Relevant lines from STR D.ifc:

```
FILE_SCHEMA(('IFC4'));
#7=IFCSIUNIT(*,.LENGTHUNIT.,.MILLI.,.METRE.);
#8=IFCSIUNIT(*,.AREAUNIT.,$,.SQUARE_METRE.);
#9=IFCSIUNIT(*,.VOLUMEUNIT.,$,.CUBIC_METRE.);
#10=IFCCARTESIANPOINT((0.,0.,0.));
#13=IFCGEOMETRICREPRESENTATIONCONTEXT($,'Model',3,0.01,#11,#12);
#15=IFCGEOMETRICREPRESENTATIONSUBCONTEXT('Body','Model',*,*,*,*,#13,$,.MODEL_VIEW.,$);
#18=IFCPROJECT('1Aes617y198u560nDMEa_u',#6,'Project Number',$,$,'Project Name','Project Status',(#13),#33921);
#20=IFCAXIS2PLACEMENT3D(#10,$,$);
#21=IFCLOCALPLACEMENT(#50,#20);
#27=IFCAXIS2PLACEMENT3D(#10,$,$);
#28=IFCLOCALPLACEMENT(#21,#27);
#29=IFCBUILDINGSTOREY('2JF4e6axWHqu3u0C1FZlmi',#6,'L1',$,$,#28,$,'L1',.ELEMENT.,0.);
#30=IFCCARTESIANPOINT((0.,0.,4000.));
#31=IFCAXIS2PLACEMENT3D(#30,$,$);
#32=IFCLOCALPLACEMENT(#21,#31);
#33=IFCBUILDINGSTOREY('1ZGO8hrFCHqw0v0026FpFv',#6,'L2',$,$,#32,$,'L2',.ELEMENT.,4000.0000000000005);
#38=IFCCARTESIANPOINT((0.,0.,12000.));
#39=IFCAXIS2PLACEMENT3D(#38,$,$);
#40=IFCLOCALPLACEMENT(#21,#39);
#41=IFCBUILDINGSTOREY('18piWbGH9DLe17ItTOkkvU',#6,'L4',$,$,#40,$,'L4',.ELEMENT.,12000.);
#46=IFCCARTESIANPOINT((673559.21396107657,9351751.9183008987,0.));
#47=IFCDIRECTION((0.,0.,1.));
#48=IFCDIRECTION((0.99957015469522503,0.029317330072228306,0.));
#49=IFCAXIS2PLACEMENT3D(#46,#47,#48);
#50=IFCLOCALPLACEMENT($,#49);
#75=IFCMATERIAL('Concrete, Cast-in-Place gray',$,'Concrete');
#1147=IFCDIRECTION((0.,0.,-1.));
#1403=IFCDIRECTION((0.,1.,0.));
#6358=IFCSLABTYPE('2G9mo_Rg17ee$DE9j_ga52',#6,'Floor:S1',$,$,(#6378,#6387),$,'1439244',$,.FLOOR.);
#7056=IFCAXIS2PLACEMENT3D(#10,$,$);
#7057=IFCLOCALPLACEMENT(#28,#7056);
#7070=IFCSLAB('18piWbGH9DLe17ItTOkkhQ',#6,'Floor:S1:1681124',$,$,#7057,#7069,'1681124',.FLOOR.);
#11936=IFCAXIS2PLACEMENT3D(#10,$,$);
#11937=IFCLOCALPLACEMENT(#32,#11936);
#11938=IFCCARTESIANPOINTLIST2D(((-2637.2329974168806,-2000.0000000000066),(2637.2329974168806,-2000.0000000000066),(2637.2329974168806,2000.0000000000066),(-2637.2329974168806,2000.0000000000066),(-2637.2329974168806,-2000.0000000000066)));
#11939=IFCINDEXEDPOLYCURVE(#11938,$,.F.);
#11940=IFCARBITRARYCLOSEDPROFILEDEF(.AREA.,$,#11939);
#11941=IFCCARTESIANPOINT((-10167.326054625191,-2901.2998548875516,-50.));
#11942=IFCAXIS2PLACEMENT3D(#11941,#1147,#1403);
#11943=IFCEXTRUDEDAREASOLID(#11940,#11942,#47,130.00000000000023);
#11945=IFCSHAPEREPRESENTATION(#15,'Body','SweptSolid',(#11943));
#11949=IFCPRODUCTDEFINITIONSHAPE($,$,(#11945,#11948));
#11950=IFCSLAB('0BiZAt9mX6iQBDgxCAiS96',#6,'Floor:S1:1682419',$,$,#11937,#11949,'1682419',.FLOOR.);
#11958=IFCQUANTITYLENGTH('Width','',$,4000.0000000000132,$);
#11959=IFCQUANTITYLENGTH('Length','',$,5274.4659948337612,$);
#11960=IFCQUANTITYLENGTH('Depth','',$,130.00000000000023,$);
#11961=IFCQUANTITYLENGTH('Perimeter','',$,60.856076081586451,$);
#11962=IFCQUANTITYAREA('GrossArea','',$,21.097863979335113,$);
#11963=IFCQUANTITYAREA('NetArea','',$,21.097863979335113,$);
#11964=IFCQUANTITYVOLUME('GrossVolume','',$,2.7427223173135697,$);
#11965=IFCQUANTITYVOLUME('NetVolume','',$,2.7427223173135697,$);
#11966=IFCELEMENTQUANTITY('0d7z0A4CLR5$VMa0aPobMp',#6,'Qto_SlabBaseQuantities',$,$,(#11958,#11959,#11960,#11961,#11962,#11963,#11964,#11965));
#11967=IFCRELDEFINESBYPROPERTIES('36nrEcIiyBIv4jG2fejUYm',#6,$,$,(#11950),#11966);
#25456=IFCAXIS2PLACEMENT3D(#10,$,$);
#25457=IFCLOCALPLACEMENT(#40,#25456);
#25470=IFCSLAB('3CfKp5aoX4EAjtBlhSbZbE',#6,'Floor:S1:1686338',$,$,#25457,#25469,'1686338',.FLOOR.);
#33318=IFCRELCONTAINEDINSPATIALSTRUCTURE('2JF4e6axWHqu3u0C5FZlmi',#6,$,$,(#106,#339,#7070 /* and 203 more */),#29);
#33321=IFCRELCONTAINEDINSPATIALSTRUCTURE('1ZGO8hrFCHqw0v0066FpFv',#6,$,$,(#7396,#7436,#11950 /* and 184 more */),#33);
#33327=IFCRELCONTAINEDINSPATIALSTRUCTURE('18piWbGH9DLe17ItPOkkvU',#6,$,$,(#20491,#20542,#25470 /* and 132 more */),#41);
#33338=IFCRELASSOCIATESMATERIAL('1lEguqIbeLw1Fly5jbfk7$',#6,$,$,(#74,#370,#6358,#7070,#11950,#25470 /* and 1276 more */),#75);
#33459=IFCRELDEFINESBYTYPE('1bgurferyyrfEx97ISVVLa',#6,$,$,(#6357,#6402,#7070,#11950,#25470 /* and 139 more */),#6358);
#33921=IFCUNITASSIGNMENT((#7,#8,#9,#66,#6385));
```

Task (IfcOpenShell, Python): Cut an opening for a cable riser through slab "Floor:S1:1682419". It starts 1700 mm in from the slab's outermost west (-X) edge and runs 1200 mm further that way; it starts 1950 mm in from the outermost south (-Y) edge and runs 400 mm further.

```python
import numpy as np
import ifcopenshell
import ifcopenshell.api.feature
import ifcopenshell.api.geometry
import ifcopenshell.api.pset
import ifcopenshell.api.root
import ifcopenshell.geom
import ifcopenshell.util.element
import ifcopenshell.util.placement
import ifcopenshell.util.representation
import ifcopenshell.util.shape
import ifcopenshell.util.unit

model = ifcopenshell.open("STR D.ifc")
unit_scale = ifcopenshell.util.unit.calculate_unit_scale(model)
area_scale = ifcopenshell.util.unit.calculate_unit_scale(model, "AREAUNIT")
volume_scale = ifcopenshell.util.unit.calculate_unit_scale(model, "VOLUMEUNIT")
settings = ifcopenshell.geom.settings()


def volume(element):
    """Net volume in cubic metres, openings subtracted."""
    shape = ifcopenshell.geom.create_shape(settings, element)
    return ifcopenshell.util.shape.get_volume(shape.geometry)


slab = model.by_id(11950)
before = volume(slab)

# Extent in the slab's own axes, in metres. The edges named are its -X and -Y sides.
slab_shape = ifcopenshell.geom.create_shape(settings, slab)
vertices = ifcopenshell.util.shape.get_vertices(slab_shape.geometry)
x_min, y_min, bottom = vertices.min(axis=0)
top = vertices[:, 2].max()

opening = ifcopenshell.api.root.create_entity(model, ifc_class="IfcOpeningElement", name="Cable riser opening", predefined_type="OPENING")
context = ifcopenshell.util.representation.get_context(model, "Model", "Body", "MODEL_VIEW")
width, depth = 1.2, 0.4
outline = [(0.0, 0.0), (width, 0.0), (width, depth), (0.0, depth), (0.0, 0.0)]
# Overshoot both faces by 50 mm so the cut is clean.
shape = ifcopenshell.api.geometry.add_slab_representation(
    model, context=context, depth=top - bottom + 0.1, polyline=outline
)
ifcopenshell.api.geometry.assign_representation(model, product=opening, representation=shape)

matrix = ifcopenshell.util.placement.get_local_placement(slab.ObjectPlacement)
matrix[:, 3] = matrix @ np.append(np.array([x_min + 1.7, y_min + 1.95, bottom - 0.05]) / unit_scale, 1.0)
ifcopenshell.api.geometry.edit_object_placement(model, product=opening, matrix=matrix, is_si=False)
ifcopenshell.api.feature.add_feature(model, feature=opening, element=slab)

after = volume(slab)

# Update the slab's stored quantities.
qto = model.by_id(ifcopenshell.util.element.get_pset(slab, "Qto_SlabBaseQuantities", should_inherit=False)["id"])
ifcopenshell.api.pset.edit_qto(model, qto=qto, properties={
    "NetArea": after / (top - bottom) / area_scale,
    "NetVolume": after / volume_scale,
})

print(f"slab volume {before:.3f} -> {after:.3f} m3")

model.write("STR D-out.ifc")
```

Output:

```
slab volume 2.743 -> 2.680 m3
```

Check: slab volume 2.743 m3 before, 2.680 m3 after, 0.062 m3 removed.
